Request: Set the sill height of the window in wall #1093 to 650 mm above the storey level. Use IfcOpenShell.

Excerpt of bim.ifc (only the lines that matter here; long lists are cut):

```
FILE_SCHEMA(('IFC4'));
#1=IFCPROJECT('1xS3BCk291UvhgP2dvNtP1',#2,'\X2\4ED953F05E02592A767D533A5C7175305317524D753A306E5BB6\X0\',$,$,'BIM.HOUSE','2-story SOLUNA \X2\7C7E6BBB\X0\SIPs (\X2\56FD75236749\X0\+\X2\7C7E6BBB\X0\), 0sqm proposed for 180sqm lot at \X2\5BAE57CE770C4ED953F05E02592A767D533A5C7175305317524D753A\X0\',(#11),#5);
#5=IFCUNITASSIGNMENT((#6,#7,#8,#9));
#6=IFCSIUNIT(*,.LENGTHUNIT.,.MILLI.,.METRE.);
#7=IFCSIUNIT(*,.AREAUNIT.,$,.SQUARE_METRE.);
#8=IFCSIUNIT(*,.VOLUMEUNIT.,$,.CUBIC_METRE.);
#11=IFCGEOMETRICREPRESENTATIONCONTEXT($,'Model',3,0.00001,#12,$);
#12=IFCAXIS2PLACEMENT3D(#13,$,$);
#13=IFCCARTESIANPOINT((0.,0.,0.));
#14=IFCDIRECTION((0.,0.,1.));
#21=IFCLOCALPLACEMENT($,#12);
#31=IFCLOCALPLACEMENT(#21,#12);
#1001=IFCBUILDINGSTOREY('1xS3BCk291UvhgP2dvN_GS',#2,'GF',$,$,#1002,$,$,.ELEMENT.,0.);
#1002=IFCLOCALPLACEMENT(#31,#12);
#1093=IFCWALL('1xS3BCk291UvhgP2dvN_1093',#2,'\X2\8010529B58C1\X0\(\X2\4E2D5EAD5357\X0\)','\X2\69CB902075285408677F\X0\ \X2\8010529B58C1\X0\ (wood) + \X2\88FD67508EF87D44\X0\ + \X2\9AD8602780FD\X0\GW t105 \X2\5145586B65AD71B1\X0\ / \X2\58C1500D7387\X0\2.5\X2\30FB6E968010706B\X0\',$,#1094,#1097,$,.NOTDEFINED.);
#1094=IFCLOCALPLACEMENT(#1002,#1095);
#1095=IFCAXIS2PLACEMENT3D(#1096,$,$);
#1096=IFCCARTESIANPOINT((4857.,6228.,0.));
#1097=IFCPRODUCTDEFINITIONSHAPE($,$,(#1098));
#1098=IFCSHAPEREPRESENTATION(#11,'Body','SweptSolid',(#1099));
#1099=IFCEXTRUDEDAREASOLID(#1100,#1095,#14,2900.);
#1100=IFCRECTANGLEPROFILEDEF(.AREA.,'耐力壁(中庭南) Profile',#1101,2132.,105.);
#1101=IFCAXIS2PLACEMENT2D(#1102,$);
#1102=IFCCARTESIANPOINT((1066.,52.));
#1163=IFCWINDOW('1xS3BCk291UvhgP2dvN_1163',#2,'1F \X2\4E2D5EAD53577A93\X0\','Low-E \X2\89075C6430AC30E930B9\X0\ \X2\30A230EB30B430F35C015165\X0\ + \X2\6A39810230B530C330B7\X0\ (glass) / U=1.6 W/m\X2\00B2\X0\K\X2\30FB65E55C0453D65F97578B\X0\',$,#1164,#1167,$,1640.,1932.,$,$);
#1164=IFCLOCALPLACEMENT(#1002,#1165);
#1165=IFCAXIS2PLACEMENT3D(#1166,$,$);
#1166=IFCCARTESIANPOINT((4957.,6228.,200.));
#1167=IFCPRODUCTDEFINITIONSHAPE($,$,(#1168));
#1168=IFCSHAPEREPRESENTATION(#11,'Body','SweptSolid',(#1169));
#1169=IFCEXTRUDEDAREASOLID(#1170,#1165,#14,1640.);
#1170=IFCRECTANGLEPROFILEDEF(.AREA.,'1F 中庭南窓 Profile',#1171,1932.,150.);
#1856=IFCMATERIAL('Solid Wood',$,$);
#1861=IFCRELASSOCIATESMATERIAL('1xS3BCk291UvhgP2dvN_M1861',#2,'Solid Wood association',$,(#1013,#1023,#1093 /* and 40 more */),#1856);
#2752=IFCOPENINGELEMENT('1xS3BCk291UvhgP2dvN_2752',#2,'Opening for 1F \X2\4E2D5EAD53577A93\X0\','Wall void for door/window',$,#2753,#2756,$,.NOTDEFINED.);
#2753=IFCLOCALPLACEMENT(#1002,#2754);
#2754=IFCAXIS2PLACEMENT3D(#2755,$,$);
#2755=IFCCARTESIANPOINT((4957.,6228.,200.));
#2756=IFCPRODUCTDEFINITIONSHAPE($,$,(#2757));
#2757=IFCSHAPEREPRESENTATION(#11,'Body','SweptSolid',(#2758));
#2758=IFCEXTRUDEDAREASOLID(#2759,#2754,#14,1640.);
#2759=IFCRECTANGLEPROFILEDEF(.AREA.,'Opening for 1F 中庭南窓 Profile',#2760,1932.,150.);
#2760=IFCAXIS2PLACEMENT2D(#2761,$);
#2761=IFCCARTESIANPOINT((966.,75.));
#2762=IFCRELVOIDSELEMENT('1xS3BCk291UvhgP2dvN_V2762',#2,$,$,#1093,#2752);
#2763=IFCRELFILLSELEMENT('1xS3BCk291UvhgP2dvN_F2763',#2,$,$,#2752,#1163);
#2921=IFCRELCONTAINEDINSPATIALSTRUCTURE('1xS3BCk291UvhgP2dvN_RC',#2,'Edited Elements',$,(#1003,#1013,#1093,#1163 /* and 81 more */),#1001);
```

```python
import numpy as np
import ifcopenshell
import ifcopenshell.api.geometry
import ifcopenshell.geom
import ifcopenshell.util.element
import ifcopenshell.util.placement
import ifcopenshell.util.shape
import ifcopenshell.util.unit

model = ifcopenshell.open("bim.ifc")
unit_scale = ifcopenshell.util.unit.calculate_unit_scale(model)

window = model.by_guid("1xS3BCk291UvhgP2dvN_1163")
opening = window.FillsVoids[0].RelatingOpeningElement
storey = ifcopenshell.util.element.get_container(window, ifc_class="IfcBuildingStorey")
level = ifcopenshell.util.placement.get_local_placement(storey.ObjectPlacement)[2, 3]

# The opening's origin need not be at the sill, so measure its lowest point.
shape = ifcopenshell.geom.create_shape(ifcopenshell.geom.settings(), opening)
bottom = ifcopenshell.util.shape.get_shape_bottom_elevation(shape, shape.geometry) / unit_scale
dz = level + 0.65 / unit_scale - bottom

shift = np.array([0.0, 0.0, dz])
# The window is not placed relative to its opening, so move both.
for product in (opening, window):
    matrix = ifcopenshell.util.placement.get_local_placement(product.ObjectPlacement)
    matrix[:3, 3] += shift
    ifcopenshell.api.geometry.edit_object_placement(model, product=product, matrix=matrix, is_si=False)

print(f"moved by {dz * unit_scale:+.3f} m")

model.write("bim_updated.ifc")
```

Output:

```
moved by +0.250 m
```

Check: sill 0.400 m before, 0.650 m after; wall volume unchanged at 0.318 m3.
